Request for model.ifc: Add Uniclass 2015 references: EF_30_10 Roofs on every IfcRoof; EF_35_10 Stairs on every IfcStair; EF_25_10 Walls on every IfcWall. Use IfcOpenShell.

First a look at what the model holds.

```python
import ifcopenshell

model = ifcopenshell.open("model.ifc")
print(model.schema)
print("classifications:", [c.Name for c in model.by_type("IfcClassification")])
for ifc_class in ("IfcDoor", "IfcRoof", "IfcStair", "IfcWall", "IfcWindow"):
    print(ifc_class, len(model.by_type(ifc_class)))
```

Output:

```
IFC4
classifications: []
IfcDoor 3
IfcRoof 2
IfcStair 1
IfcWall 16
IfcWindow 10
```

```python
import ifcopenshell
import ifcopenshell.api.classification

model = ifcopenshell.open("model.ifc")

system = ifcopenshell.api.classification.add_classification(model, classification="Uniclass 2015")

codes = {
    "IfcRoof": ("EF_30_10", "Roofs"),
    "IfcStair": ("EF_35_10", "Stairs"),
    "IfcWall": ("EF_25_10", "Walls"),
}
for ifc_class, (code, name) in codes.items():
    products = model.by_type(ifc_class)
    ifcopenshell.api.classification.add_reference(
        model, products=products, classification=system, identification=code, name=name
    )
    print(code, len(products))

model.write("model_rev.ifc")
```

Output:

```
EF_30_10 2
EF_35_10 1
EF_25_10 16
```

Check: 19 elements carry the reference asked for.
